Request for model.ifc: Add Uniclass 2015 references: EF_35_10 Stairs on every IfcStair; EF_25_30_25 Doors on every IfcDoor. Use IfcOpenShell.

First a look at what the model holds.

```python
import ifcopenshell

model = ifcopenshell.open("model.ifc")
print(model.schema)
print("classifications:", [c.Name for c in model.by_type("IfcClassification")])
for ifc_class in ("IfcDoor", "IfcRoof", "IfcStair", "IfcWall", "IfcWindow"):
    print(ifc_class, len(model.by_type(ifc_class)))
```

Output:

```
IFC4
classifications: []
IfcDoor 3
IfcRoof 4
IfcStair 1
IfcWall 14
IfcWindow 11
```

```python
import ifcopenshell
import ifcopenshell.api.classification

model = ifcopenshell.open("model.ifc")

system = ifcopenshell.api.classification.add_classification(model, classification="Uniclass 2015")

codes = {
    "IfcStair": ("EF_35_10", "Stairs"),
    "IfcDoor": ("EF_25_30_25", "Doors"),
}
for ifc_class, (code, name) in codes.items():
    products = model.by_type(ifc_class)
    ifcopenshell.api.classification.add_reference(
        model, products=products, classification=system, identification=code, name=name
    )
    print(code, len(products))

model.write("model_edited.ifc")
```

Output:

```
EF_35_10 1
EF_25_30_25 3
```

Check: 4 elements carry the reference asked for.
